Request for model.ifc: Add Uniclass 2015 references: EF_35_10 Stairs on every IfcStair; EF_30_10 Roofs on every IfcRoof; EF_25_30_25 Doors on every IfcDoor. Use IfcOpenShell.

First a look at what the model holds.

```python
import ifcopenshell

model = ifcopenshell.open("model.ifc")
print(model.schema)
print("classifications:", [c.Name for c in model.by_type("IfcClassification")])
for ifc_class in ("IfcDoor", "IfcRoof", "IfcStair", "IfcWall", "IfcWindow"):
    print(ifc_class, len(model.by_type(ifc_class)))
```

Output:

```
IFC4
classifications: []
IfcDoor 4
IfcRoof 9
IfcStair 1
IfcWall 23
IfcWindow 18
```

```python
import ifcopenshell
import ifcopenshell.api.classification

model = ifcopenshell.open("model.ifc")

system = ifcopenshell.api.classification.add_classification(model, classification="Uniclass 2015")

codes = {
    "IfcStair": ("EF_35_10", "Stairs"),
    "IfcRoof": ("EF_30_10", "Roofs"),
    "IfcDoor": ("EF_25_30_25", "Doors"),
}
for ifc_class, (code, name) in codes.items():
    products = model.by_type(ifc_class)
    ifcopenshell.api.classification.add_reference(
        model, products=products, classification=system, identification=code, name=name
    )
    print(code, len(products))

model.write("model-out.ifc")
```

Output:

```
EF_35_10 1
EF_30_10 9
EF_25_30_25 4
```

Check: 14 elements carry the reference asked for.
